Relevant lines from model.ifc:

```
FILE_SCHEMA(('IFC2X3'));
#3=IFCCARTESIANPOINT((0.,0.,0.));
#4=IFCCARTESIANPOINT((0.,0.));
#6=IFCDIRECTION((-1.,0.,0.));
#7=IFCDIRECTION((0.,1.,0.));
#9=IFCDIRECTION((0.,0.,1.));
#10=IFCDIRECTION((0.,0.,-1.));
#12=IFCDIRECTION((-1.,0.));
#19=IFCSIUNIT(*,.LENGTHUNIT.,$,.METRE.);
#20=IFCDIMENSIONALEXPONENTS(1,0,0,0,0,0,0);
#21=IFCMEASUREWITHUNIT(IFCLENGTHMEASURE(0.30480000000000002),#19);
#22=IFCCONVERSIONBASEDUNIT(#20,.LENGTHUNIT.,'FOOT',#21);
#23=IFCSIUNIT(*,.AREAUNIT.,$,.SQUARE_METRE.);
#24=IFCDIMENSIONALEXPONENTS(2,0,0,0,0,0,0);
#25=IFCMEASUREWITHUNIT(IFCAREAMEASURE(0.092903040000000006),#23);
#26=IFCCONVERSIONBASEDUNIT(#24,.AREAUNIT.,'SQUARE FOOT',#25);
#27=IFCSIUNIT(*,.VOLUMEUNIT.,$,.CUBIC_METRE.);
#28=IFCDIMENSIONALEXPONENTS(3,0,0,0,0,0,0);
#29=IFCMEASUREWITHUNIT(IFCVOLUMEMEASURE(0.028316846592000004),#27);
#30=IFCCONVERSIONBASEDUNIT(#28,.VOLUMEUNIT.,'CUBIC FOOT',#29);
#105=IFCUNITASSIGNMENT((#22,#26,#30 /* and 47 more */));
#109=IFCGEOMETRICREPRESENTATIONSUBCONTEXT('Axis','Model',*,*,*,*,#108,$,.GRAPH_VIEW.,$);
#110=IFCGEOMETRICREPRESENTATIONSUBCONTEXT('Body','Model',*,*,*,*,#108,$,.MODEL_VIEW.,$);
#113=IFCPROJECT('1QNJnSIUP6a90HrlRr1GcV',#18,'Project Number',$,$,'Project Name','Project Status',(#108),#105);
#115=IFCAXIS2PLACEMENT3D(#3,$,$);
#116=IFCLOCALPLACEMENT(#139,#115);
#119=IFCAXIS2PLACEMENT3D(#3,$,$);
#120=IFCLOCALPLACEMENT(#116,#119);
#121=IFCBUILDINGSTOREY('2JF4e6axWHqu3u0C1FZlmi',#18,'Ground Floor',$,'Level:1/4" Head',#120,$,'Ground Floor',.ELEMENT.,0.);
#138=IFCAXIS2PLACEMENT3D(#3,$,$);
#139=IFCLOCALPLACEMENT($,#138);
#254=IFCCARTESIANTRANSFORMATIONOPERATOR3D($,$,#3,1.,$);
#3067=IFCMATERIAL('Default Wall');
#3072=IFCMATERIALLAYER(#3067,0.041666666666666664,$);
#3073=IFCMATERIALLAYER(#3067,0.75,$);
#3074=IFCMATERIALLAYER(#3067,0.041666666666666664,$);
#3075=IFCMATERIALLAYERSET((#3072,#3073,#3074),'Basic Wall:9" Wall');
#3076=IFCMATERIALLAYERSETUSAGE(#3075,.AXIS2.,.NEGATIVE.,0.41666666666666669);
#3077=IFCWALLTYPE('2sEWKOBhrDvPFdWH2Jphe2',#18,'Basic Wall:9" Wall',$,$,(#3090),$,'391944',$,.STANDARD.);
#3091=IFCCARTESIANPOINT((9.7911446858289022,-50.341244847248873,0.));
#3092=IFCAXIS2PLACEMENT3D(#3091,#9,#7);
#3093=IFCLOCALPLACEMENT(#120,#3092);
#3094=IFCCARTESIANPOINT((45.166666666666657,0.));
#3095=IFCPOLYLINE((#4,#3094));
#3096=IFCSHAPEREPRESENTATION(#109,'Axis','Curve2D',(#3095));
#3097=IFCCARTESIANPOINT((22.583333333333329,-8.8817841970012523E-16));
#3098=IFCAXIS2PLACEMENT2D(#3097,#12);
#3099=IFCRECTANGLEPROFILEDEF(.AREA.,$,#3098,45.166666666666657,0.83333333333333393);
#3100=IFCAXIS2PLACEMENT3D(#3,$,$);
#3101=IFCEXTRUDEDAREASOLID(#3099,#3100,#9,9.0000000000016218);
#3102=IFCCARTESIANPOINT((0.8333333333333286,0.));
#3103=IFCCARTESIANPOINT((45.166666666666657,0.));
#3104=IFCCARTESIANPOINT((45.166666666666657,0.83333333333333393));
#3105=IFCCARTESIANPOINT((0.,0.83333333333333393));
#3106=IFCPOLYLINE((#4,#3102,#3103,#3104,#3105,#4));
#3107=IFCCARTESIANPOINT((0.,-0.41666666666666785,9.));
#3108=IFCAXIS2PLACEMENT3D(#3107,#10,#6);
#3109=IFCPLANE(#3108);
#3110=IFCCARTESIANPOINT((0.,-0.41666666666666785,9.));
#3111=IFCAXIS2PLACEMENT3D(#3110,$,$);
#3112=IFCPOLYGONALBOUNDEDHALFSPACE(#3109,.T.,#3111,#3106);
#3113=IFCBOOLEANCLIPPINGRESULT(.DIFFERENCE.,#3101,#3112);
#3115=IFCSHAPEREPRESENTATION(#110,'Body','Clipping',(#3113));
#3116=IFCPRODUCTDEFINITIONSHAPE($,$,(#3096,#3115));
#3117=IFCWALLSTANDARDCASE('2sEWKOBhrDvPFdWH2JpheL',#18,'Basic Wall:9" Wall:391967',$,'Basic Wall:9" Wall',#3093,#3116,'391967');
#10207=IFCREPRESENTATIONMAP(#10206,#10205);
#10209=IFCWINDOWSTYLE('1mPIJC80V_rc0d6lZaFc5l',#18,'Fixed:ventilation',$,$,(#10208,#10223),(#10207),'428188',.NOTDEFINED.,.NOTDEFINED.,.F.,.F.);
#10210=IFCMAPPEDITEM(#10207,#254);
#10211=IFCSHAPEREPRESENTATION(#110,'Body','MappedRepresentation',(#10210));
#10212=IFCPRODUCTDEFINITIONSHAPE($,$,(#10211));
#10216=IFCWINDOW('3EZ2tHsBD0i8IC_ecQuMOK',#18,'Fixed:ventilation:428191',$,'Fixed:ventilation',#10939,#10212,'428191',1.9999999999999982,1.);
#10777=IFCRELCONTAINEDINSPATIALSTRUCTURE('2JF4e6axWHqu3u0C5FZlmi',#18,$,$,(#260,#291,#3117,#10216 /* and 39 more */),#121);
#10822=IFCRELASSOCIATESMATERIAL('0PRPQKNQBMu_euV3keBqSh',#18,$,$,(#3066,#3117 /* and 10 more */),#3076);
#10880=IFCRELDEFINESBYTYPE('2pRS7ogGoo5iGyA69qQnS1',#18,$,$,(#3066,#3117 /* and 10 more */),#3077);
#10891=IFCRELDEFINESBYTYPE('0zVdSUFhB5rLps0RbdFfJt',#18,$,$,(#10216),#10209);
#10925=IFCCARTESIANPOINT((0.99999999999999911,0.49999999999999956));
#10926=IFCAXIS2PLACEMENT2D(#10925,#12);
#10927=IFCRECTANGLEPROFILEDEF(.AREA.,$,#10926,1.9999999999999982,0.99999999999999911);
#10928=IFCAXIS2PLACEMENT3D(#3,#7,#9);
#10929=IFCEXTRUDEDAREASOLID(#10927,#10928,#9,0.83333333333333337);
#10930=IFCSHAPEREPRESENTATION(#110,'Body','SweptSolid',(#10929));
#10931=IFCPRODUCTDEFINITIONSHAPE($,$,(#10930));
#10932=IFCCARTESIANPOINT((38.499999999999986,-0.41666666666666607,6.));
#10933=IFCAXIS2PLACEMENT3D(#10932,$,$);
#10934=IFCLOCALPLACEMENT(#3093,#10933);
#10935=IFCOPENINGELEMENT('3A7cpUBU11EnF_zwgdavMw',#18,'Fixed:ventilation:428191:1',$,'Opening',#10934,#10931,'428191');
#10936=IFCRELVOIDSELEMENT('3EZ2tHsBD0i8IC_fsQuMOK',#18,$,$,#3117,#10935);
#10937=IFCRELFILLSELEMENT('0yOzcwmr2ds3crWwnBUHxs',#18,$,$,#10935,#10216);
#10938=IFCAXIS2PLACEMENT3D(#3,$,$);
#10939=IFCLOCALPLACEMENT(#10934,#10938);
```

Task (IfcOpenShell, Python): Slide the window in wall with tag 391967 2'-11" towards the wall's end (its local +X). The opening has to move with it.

```python
import ifcopenshell
import ifcopenshell.api.geometry
import ifcopenshell.util.placement
import ifcopenshell.util.unit

model = ifcopenshell.open("model.ifc")
unit_scale = ifcopenshell.util.unit.calculate_unit_scale(model)

window = model.by_guid("3EZ2tHsBD0i8IC_ecQuMOK")
opening = window.FillsVoids[0].RelatingOpeningElement
wall = opening.VoidsElements[0].RelatingBuildingElement

wall_matrix = ifcopenshell.util.placement.get_local_placement(wall.ObjectPlacement)
shift = wall_matrix[:3, 0] * 35 * 0.0254 / unit_scale
before = ifcopenshell.util.placement.get_local_placement(window.ObjectPlacement)[:3, 3].copy()

# The window is placed relative to its opening, so it follows when the opening moves.
matrix = ifcopenshell.util.placement.get_local_placement(opening.ObjectPlacement)
matrix[:3, 3] += shift
ifcopenshell.api.geometry.edit_object_placement(
    model, product=opening, matrix=matrix, is_si=False, should_transform_children=True
)

after = ifcopenshell.util.placement.get_local_placement(window.ObjectPlacement)[:3, 3]
print("window moved by", (after - before).round(3) + 0.0)

model.write("model_edited.ifc")
```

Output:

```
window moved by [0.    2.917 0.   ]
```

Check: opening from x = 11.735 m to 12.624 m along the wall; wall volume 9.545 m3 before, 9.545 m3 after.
